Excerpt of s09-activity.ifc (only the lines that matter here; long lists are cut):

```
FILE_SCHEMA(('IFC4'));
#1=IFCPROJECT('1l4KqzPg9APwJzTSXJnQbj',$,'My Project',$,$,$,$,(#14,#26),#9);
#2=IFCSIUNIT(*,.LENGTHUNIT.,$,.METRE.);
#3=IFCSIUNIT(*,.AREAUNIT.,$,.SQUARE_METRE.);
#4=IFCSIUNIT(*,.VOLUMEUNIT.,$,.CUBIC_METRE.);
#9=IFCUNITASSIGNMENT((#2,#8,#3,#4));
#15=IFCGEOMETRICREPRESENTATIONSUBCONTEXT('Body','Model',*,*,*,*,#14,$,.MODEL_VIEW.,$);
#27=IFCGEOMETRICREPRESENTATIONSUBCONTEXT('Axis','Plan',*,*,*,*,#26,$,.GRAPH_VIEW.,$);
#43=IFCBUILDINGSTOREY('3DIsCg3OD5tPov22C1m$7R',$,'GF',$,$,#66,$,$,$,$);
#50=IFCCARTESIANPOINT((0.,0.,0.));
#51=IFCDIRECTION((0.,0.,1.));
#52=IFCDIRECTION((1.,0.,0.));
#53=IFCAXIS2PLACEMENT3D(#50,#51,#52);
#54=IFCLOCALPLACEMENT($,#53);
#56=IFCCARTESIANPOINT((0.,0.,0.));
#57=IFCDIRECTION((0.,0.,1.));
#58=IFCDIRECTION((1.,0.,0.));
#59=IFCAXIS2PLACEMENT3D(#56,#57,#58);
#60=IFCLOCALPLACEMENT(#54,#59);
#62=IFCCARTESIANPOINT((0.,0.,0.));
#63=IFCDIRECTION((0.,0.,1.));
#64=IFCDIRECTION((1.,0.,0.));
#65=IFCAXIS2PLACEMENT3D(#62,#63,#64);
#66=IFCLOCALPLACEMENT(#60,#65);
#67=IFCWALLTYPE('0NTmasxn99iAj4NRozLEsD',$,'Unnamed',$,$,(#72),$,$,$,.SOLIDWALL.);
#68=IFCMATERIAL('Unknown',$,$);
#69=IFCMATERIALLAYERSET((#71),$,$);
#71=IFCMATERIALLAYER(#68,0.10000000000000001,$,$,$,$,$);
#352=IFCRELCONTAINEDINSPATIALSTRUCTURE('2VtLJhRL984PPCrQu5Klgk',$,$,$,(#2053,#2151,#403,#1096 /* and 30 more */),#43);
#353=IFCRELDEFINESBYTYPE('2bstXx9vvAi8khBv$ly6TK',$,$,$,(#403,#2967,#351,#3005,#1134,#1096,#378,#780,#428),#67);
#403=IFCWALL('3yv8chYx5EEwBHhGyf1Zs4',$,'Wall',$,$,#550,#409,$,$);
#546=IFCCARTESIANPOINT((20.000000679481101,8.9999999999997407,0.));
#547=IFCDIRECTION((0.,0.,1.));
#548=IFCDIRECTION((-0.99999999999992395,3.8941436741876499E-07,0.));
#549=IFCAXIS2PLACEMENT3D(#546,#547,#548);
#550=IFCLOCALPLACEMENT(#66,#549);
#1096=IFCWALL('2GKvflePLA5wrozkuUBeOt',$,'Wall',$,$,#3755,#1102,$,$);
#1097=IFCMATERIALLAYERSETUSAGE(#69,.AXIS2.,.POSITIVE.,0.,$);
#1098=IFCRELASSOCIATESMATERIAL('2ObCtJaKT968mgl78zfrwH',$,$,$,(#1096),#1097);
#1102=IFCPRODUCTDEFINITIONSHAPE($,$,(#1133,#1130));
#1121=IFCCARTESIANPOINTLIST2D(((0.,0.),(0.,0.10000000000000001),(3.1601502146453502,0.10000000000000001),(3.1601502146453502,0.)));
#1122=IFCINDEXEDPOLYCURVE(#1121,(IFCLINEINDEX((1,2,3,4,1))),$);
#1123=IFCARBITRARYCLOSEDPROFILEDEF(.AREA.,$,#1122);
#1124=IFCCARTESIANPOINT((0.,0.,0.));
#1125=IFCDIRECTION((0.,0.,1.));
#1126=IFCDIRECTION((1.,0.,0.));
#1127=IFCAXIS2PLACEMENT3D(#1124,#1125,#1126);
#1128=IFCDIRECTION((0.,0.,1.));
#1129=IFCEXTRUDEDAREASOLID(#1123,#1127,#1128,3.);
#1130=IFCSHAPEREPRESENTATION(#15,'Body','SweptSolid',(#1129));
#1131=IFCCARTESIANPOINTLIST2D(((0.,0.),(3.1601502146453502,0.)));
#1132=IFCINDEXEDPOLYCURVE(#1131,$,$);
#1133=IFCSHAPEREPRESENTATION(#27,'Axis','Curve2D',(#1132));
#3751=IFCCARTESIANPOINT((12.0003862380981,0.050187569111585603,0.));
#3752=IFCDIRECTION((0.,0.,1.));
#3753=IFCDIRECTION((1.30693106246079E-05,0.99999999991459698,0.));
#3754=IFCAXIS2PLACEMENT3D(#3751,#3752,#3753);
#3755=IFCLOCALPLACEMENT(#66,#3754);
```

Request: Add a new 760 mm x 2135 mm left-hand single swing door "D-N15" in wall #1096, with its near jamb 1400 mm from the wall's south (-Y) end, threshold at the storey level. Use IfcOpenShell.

```python
import numpy as np
import ifcopenshell
import ifcopenshell.api.feature
import ifcopenshell.api.geometry
import ifcopenshell.api.root
import ifcopenshell.api.spatial
import ifcopenshell.geom
import ifcopenshell.util.element
import ifcopenshell.util.placement
import ifcopenshell.util.representation
import ifcopenshell.util.shape
import ifcopenshell.util.unit

model = ifcopenshell.open("s09-activity.ifc")
unit_scale = ifcopenshell.util.unit.calculate_unit_scale(model)
settings = ifcopenshell.geom.settings()


def volume(element):
    """Net volume in cubic metres, openings subtracted."""
    shape = ifcopenshell.geom.create_shape(settings, element)
    return ifcopenshell.util.shape.get_volume(shape.geometry)


wall = model.by_id(1096)
storey = ifcopenshell.util.element.get_container(wall, ifc_class="IfcBuildingStorey")
context = ifcopenshell.util.representation.get_context(model, "Model", "Body", "MODEL_VIEW")
before = volume(wall)

width, height, from_end, sill = 0.76, 2.135, 1.4, 0.0  # metres

# The wall runs along its own X axis, and the end named is its -X end.
wall_shape = ifcopenshell.geom.create_shape(settings, wall)
x, y, z = ifcopenshell.util.shape.get_vertices(wall_shape.geometry).T
start = x.min() + from_end
face, thickness = float(y.min()), float(y.max() - y.min())
wall_matrix = ifcopenshell.util.placement.get_local_placement(wall.ObjectPlacement)
level = ifcopenshell.util.placement.get_local_placement(storey.ObjectPlacement)[2, 3]


def in_wall(x, y):
    """Placement at x, y metres in the wall's axes, at sill height."""
    matrix = wall_matrix.copy()
    matrix[:, 3] = wall_matrix @ np.array([x / unit_scale, y / unit_scale, 0.0, 1.0])
    matrix[2, 3] = level + sill / unit_scale
    return matrix


# Opening: a box that overshoots both wall faces by 50 mm.
opening = ifcopenshell.api.root.create_entity(model, ifc_class="IfcOpeningElement", predefined_type="OPENING")
box = ifcopenshell.api.geometry.add_wall_representation(
    model, context=context, length=width, height=height, thickness=thickness + 0.1
)
ifcopenshell.api.geometry.assign_representation(model, product=opening, representation=box)
ifcopenshell.api.geometry.edit_object_placement(model, product=opening, matrix=in_wall(start, face - 0.05), is_si=False)
ifcopenshell.api.feature.add_feature(model, feature=opening, element=wall)

door = ifcopenshell.api.root.create_entity(model, ifc_class="IfcDoor", name="D-N15", predefined_type="DOOR")
door.OverallWidth, door.OverallHeight = width / unit_scale, height / unit_scale
door.OperationType = "SINGLE_SWING_LEFT"
body = ifcopenshell.api.geometry.add_door_representation(
    model,
    context=context,
    overall_width=door.OverallWidth,
    overall_height=door.OverallHeight,
    operation_type="SINGLE_SWING_LEFT",
    lining_properties={"LiningDepth": thickness / unit_scale, "ThresholdDepth": thickness / unit_scale},
)
ifcopenshell.api.geometry.assign_representation(model, product=door, representation=body)
ifcopenshell.api.spatial.assign_container(model, products=[door], relating_structure=storey)
ifcopenshell.api.feature.add_filling(model, opening=opening, element=door)

# The lining spans the wall, so the door starts at the wall face.
ifcopenshell.api.geometry.edit_object_placement(model, product=door, matrix=in_wall(start, face), is_si=False)

after = volume(wall)

print(f"wall volume {before:.3f} -> {after:.3f} m3")

model.write("s09-activity-out.ifc")
```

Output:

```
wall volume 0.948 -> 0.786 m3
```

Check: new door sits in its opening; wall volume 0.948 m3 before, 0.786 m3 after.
